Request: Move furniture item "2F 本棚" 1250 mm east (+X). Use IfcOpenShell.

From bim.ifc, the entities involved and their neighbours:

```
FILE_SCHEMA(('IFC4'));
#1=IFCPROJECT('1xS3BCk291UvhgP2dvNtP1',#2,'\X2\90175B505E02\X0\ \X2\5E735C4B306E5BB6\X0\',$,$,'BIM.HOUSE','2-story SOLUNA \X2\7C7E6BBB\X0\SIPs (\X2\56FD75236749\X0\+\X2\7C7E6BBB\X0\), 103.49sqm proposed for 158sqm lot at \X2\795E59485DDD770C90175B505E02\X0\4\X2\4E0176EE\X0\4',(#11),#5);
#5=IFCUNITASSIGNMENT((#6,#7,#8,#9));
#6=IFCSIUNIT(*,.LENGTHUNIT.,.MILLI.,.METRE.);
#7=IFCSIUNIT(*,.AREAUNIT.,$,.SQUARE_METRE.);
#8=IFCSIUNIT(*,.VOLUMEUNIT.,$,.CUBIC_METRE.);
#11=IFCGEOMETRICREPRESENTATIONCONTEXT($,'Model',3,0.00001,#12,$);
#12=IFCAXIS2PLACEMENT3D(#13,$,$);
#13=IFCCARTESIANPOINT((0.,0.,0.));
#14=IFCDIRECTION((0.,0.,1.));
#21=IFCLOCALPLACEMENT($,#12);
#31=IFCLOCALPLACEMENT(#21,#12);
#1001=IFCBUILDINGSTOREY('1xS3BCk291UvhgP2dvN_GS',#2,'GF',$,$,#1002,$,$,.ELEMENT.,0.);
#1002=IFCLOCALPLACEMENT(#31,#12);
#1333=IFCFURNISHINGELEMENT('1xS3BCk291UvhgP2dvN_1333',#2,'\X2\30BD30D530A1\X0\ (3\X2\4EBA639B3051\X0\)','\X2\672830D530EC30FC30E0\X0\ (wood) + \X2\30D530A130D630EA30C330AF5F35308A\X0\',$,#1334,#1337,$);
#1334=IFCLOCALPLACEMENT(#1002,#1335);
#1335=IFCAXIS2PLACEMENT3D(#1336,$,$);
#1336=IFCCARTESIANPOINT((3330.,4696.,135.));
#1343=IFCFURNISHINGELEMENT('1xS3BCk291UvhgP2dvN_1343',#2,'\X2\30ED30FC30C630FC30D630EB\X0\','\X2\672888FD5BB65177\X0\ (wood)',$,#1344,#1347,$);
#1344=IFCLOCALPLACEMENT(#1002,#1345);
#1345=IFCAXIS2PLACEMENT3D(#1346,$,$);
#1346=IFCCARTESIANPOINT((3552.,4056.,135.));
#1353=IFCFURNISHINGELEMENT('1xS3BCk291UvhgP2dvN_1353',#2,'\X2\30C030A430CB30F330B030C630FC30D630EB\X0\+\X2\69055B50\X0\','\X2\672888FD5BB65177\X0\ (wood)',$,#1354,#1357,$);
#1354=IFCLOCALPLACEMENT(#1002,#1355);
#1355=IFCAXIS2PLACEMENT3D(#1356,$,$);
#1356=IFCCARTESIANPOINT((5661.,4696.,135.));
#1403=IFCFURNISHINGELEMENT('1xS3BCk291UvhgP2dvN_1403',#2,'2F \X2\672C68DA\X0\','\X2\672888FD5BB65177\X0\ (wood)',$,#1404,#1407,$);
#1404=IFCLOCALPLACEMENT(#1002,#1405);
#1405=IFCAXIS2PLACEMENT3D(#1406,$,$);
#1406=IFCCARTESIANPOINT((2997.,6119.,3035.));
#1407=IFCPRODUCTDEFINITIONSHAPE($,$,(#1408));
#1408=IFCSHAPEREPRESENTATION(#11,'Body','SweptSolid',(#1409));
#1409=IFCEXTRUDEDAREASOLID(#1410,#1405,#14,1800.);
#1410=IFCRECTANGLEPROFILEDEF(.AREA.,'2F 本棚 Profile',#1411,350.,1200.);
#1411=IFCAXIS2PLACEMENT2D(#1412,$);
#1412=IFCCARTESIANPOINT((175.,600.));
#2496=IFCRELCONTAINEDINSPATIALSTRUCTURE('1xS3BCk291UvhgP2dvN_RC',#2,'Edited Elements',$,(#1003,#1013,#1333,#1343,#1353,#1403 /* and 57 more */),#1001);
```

```python
import ifcopenshell
import ifcopenshell.api.geometry
import ifcopenshell.util.placement
import ifcopenshell.util.unit

model = ifcopenshell.open("bim.ifc")
unit_scale = ifcopenshell.util.unit.calculate_unit_scale(model)

item = model.by_guid("1xS3BCk291UvhgP2dvN_1403")
matrix = ifcopenshell.util.placement.get_local_placement(item.ObjectPlacement)
matrix[0, 3] += 1.25 / unit_scale
ifcopenshell.api.geometry.edit_object_placement(model, product=item, matrix=matrix, is_si=False)

print(ifcopenshell.util.placement.get_local_placement(item.ObjectPlacement).round(3) + 0.0)

model.write("bim-out.ifc")
```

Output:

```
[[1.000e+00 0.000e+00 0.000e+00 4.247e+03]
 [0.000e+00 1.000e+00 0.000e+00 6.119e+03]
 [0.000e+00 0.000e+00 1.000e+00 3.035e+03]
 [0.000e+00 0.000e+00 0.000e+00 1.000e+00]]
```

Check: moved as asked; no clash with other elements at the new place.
